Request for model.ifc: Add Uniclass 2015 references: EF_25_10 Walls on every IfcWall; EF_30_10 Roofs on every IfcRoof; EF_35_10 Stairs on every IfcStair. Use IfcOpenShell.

First a look at what the model holds.

```python
import ifcopenshell

model = ifcopenshell.open("model.ifc")
print(model.schema)
print("classifications:", [c.Name for c in model.by_type("IfcClassification")])
for ifc_class in ("IfcDoor", "IfcRoof", "IfcStair", "IfcWall", "IfcWindow"):
    print(ifc_class, len(model.by_type(ifc_class)))
```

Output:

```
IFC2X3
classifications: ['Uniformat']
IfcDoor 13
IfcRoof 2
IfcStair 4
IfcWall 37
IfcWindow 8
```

```python
import ifcopenshell
import ifcopenshell.api.classification

model = ifcopenshell.open("model.ifc")

# IFC2X3 requires Source and Edition and has no link from the project to the system.
system = model.create_entity("IfcClassification", Source="NBS", Edition="2015", Name="Uniclass 2015")

codes = {
    "IfcWall": ("EF_25_10", "Walls"),
    "IfcRoof": ("EF_30_10", "Roofs"),
    "IfcStair": ("EF_35_10", "Stairs"),
}
for ifc_class, (code, name) in codes.items():
    products = model.by_type(ifc_class)
    ifcopenshell.api.classification.add_reference(
        model, products=products, classification=system, identification=code, name=name
    )
    print(code, len(products))

model.write("model_edited.ifc")
```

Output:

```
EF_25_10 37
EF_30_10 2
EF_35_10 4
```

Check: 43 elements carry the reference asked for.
